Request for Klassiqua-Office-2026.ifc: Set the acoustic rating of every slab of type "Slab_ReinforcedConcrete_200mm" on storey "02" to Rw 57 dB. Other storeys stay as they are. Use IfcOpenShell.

First a look at what the model holds.

```python
import ifcopenshell
import ifcopenshell.util.element

model = ifcopenshell.open("Klassiqua-Office-2026.ifc")
print(model.schema)
storey = next(s for s in model.by_type("IfcBuildingStorey") if s.Name == "02")
slabs = [e for e in ifcopenshell.util.element.get_decomposition(storey) if e.is_a("IfcSlab")]
seen = {}
for e in slabs:
    element_type = ifcopenshell.util.element.get_type(e)
    key = (element_type.Name if element_type != e and element_type else None, ifcopenshell.util.element.get_pset(e, "Pset_SlabCommon", "AcousticRating"))
    seen[key] = seen.get(key, 0) + 1
for (name, value), count in sorted(seen.items(), key=str):
    print(count, "x", name, "|", value)
```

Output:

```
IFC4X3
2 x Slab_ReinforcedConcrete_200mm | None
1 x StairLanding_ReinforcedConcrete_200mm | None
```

```python
import ifcopenshell
import ifcopenshell.api.pset
import ifcopenshell.util.element

model = ifcopenshell.open("Klassiqua-Office-2026.ifc")

storey = next(s for s in model.by_type("IfcBuildingStorey") if s.Name == "02")
slabs = [e for e in ifcopenshell.util.element.get_decomposition(storey) if e.is_a("IfcSlab")]

count = 0
for e in slabs:
    element_type = ifcopenshell.util.element.get_type(e)
    if element_type in (None, e) or element_type.Name != "Slab_ReinforcedConcrete_200mm":
        continue
    # add_pset returns the element's existing set when there is one.
    pset = ifcopenshell.api.pset.add_pset(model, product=e, name="Pset_SlabCommon")
    ifcopenshell.api.pset.edit_pset(model, pset=pset, properties={"AcousticRating": "Rw 57 dB"})
    count += 1

print(count, "slabs updated")

model.write("Klassiqua-Office-2026_v2.ifc")
```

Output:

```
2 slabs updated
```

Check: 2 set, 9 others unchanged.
